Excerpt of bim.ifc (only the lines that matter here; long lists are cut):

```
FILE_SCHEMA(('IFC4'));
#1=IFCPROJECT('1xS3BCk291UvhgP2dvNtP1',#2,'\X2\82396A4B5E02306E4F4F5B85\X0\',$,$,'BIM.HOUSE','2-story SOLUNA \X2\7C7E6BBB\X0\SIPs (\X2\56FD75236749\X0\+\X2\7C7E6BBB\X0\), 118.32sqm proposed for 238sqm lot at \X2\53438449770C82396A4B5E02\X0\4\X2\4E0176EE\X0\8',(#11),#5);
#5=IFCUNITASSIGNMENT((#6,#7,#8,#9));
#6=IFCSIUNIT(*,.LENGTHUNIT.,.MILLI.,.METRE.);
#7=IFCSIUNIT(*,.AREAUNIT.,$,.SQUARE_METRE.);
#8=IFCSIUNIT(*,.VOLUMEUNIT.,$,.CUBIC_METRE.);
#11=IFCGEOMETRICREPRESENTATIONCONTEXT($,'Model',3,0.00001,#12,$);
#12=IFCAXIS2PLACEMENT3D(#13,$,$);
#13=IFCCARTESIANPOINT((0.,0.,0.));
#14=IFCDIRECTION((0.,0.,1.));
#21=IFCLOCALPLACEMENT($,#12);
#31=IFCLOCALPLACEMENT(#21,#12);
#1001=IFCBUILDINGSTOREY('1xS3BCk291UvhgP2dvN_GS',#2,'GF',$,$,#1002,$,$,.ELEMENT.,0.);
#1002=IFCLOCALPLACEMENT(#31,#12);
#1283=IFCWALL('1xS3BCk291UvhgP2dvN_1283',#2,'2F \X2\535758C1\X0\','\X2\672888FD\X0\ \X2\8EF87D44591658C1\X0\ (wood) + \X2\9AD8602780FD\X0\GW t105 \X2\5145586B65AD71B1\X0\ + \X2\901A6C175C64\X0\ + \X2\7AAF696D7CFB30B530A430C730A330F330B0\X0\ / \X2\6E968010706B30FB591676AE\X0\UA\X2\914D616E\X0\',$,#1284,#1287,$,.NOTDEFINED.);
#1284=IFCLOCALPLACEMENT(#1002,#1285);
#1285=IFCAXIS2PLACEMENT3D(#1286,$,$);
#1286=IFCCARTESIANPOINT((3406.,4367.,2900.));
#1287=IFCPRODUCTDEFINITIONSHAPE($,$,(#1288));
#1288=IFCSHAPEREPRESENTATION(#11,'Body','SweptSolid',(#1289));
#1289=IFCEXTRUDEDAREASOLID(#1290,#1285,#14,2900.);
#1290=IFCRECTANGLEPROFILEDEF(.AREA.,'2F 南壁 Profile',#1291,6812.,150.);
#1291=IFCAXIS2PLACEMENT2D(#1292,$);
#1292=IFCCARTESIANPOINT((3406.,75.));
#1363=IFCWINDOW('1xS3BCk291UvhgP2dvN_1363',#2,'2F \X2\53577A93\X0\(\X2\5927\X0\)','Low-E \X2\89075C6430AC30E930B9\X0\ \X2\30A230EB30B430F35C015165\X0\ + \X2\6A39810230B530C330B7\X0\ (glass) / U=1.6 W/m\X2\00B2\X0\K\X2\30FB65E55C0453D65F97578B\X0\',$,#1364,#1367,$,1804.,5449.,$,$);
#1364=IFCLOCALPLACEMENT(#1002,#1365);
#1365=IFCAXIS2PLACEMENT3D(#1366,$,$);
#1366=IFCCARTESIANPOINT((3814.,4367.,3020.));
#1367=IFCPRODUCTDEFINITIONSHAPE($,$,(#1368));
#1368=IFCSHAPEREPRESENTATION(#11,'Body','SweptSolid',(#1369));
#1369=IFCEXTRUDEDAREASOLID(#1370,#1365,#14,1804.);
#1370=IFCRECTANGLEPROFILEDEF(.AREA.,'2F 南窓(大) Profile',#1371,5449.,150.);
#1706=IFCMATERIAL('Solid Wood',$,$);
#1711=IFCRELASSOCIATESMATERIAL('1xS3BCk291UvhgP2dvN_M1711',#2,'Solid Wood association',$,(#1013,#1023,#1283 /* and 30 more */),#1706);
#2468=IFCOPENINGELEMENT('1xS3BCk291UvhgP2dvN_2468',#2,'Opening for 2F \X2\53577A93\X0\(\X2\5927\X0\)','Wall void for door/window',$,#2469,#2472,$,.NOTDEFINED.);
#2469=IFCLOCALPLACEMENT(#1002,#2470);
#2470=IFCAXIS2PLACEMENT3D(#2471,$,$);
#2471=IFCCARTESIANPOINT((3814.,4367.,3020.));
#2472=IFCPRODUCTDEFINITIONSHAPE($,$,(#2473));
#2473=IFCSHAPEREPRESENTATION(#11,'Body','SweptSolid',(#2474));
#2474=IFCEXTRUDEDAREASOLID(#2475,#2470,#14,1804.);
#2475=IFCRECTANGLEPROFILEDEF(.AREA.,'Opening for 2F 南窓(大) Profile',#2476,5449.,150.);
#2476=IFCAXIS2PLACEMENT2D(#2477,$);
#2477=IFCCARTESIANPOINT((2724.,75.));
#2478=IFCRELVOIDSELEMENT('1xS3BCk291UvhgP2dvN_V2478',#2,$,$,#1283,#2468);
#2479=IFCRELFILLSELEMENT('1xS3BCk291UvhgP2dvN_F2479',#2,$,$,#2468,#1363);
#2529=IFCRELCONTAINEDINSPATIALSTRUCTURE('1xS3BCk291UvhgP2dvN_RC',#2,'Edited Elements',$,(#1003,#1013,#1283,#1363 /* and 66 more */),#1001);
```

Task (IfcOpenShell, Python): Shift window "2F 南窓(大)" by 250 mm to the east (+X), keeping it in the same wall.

```python
import ifcopenshell
import ifcopenshell.api.geometry
import ifcopenshell.util.placement
import ifcopenshell.util.unit

model = ifcopenshell.open("bim.ifc")
unit_scale = ifcopenshell.util.unit.calculate_unit_scale(model)

window = model.by_id(1363)
opening = window.FillsVoids[0].RelatingOpeningElement
wall = opening.VoidsElements[0].RelatingBuildingElement

wall_matrix = ifcopenshell.util.placement.get_local_placement(wall.ObjectPlacement)
shift = wall_matrix[:3, 0] * 0.25 / unit_scale
before = ifcopenshell.util.placement.get_local_placement(window.ObjectPlacement)[:3, 3].copy()

# The window is not placed relative to its opening, so move both.
for product in (opening, window):
    matrix = ifcopenshell.util.placement.get_local_placement(product.ObjectPlacement)
    matrix[:3, 3] += shift
    ifcopenshell.api.geometry.edit_object_placement(model, product=product, matrix=matrix, is_si=False)

after = ifcopenshell.util.placement.get_local_placement(window.ObjectPlacement)[:3, 3]
print("window moved by", (after - before).round(3) + 0.0)

model.write("bim-out.ifc")
```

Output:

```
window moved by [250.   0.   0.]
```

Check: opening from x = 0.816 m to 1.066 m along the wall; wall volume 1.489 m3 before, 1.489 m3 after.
